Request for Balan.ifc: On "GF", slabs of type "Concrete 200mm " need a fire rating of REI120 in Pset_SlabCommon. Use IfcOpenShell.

First a look at what the model holds.

```python
import ifcopenshell
import ifcopenshell.util.element

model = ifcopenshell.open("Balan.ifc")
print(model.schema)
storey = next(s for s in model.by_type("IfcBuildingStorey") if s.Name == "GF")
slabs = [e for e in ifcopenshell.util.element.get_decomposition(storey) if e.is_a("IfcSlab")]
seen = {}
for e in slabs:
    element_type = ifcopenshell.util.element.get_type(e)
    key = (element_type.Name if element_type != e and element_type else None, ifcopenshell.util.element.get_pset(e, "Pset_SlabCommon", "FireRating"))
    seen[key] = seen.get(key, 0) + 1
for (name, value), count in sorted(seen.items(), key=str):
    print(count, "x", name, "|", value)
```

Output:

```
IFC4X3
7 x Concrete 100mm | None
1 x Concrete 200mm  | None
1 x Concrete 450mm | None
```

```python
import ifcopenshell
import ifcopenshell.api.pset
import ifcopenshell.util.element

model = ifcopenshell.open("Balan.ifc")

storey = next(s for s in model.by_type("IfcBuildingStorey") if s.Name == "GF")
slabs = [e for e in ifcopenshell.util.element.get_decomposition(storey) if e.is_a("IfcSlab")]

count = 0
for e in slabs:
    element_type = ifcopenshell.util.element.get_type(e)
    if element_type in (None, e) or element_type.Name != "Concrete 200mm ":
        continue
    # add_pset returns the element's existing set when there is one.
    pset = ifcopenshell.api.pset.add_pset(model, product=e, name="Pset_SlabCommon")
    ifcopenshell.api.pset.edit_pset(model, pset=pset, properties={"FireRating": "REI120"})
    count += 1

print(count, "slabs updated")

model.write("Balan_edited.ifc")
```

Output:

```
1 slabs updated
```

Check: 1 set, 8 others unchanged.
